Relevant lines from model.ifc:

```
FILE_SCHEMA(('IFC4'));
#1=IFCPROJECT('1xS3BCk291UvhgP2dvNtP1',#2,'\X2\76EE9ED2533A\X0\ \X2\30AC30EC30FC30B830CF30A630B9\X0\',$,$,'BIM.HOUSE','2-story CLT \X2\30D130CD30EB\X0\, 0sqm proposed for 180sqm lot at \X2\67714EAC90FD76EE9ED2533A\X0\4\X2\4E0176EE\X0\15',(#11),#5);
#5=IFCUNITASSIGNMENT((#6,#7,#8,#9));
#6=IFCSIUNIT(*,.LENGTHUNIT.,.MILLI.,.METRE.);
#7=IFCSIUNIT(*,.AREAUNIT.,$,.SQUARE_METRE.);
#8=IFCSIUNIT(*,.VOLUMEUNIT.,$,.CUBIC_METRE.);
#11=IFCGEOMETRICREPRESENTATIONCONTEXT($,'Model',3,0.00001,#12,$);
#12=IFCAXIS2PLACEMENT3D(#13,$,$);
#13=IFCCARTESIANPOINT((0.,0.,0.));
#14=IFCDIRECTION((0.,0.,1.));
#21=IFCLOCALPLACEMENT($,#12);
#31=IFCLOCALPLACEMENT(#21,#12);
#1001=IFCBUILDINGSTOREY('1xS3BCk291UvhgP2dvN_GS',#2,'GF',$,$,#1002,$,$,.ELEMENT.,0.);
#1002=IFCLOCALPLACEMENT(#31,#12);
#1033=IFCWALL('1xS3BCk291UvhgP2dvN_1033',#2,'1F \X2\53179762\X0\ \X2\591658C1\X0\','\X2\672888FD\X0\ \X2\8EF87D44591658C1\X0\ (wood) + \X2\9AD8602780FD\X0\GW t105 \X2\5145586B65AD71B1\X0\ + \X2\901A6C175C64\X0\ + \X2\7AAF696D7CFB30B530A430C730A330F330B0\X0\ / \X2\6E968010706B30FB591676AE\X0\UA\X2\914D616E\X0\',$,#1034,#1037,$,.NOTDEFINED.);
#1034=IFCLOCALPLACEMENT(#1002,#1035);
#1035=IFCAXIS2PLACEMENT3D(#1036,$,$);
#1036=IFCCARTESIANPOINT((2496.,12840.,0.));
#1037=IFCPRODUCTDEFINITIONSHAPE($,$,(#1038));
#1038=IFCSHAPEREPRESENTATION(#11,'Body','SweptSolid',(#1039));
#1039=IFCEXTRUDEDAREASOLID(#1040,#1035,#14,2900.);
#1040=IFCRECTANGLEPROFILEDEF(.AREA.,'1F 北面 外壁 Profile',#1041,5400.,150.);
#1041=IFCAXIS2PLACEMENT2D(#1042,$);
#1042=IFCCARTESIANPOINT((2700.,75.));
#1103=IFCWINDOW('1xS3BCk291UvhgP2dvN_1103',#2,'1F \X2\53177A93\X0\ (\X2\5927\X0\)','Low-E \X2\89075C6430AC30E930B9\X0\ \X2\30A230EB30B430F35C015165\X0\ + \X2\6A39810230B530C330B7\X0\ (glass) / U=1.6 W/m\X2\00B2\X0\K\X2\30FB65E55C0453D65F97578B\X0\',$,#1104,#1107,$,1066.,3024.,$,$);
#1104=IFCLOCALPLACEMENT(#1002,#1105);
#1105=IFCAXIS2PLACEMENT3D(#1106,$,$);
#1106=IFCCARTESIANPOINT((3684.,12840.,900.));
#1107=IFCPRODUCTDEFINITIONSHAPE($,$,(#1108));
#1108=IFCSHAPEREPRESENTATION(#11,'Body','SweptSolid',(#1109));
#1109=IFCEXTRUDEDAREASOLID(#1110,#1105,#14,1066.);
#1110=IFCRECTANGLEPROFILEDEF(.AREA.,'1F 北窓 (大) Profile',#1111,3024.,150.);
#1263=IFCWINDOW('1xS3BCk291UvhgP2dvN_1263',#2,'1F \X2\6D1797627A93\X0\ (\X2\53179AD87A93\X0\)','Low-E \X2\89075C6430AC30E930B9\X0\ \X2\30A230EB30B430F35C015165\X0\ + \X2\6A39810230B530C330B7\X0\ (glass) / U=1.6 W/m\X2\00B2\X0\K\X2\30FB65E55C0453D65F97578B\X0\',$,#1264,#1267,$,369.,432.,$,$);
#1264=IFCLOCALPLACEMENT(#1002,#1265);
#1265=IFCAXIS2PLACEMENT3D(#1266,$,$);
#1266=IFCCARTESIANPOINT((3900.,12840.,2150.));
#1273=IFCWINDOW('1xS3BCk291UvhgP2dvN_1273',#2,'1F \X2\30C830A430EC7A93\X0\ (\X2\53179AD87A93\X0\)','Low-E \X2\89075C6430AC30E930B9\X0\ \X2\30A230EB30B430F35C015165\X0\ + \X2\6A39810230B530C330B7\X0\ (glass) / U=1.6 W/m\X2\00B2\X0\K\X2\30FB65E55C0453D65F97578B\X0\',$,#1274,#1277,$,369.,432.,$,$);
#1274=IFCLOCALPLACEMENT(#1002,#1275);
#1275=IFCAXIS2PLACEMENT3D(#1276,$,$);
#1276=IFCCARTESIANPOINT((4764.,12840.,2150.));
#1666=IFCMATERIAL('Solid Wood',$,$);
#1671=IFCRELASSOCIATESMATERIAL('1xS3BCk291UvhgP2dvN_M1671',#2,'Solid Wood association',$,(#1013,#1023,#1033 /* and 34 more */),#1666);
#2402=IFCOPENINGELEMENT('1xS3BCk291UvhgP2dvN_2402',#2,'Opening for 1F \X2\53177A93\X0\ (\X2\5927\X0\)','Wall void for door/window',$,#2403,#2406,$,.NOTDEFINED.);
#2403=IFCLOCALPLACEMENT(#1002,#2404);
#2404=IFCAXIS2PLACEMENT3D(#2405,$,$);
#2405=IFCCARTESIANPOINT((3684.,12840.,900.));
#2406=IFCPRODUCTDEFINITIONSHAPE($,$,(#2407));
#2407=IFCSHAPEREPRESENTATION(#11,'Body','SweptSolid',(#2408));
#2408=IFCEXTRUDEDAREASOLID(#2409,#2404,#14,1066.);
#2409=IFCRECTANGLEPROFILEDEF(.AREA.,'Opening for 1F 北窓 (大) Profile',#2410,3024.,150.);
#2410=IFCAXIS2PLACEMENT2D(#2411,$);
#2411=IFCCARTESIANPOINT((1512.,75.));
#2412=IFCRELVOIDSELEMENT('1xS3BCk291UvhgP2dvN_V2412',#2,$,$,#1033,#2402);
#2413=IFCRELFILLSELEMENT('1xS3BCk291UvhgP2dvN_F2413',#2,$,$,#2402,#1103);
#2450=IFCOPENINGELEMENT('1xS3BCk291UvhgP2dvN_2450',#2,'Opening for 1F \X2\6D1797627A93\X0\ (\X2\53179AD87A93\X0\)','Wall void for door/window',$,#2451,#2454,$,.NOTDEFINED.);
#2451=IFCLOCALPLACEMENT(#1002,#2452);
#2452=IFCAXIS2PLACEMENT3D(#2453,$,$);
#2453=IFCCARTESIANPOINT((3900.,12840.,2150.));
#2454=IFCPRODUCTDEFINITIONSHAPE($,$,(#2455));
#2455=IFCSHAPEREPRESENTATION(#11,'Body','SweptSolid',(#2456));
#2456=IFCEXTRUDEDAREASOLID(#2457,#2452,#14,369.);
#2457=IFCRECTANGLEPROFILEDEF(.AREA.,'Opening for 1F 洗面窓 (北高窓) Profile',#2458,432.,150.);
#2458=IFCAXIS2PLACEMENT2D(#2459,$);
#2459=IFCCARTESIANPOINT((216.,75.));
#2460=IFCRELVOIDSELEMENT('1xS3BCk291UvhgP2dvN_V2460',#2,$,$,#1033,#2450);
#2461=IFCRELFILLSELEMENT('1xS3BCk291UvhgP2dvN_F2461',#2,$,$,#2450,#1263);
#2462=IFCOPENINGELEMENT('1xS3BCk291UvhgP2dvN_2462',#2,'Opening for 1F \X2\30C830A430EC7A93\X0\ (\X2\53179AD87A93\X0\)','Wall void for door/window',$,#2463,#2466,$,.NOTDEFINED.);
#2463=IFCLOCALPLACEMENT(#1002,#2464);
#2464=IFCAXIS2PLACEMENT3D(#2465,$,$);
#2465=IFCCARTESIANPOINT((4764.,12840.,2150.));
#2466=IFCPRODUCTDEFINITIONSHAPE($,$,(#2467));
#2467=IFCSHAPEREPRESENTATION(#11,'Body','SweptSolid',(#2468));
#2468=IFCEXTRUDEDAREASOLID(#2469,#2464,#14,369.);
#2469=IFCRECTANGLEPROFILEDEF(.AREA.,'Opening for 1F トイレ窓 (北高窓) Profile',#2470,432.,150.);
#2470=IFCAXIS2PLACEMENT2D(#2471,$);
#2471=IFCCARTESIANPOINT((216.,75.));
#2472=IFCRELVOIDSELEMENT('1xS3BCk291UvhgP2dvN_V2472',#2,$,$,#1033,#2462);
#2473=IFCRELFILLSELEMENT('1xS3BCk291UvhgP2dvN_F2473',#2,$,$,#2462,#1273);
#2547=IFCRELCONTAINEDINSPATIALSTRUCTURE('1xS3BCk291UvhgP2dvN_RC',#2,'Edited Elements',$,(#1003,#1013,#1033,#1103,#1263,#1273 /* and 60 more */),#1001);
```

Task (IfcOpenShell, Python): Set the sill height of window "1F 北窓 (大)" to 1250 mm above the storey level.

```python
import numpy as np
import ifcopenshell
import ifcopenshell.api.geometry
import ifcopenshell.geom
import ifcopenshell.util.element
import ifcopenshell.util.placement
import ifcopenshell.util.shape
import ifcopenshell.util.unit

model = ifcopenshell.open("model.ifc")
unit_scale = ifcopenshell.util.unit.calculate_unit_scale(model)

window = model.by_guid("1xS3BCk291UvhgP2dvN_1103")
opening = window.FillsVoids[0].RelatingOpeningElement
storey = ifcopenshell.util.element.get_container(window, ifc_class="IfcBuildingStorey")
level = ifcopenshell.util.placement.get_local_placement(storey.ObjectPlacement)[2, 3]

# The opening's origin need not be at the sill, so measure its lowest point.
shape = ifcopenshell.geom.create_shape(ifcopenshell.geom.settings(), opening)
bottom = ifcopenshell.util.shape.get_shape_bottom_elevation(shape, shape.geometry) / unit_scale
dz = level + 1250.0 - bottom

shift = np.array([0.0, 0.0, dz])
# The window is not placed relative to its opening, so move both.
for product in (opening, window):
    matrix = ifcopenshell.util.placement.get_local_placement(product.ObjectPlacement)
    matrix[:3, 3] += shift
    ifcopenshell.api.geometry.edit_object_placement(model, product=product, matrix=matrix, is_si=False)

print(f"moved by {dz * unit_scale:+.3f} m")

model.write("model_v2.ifc")
```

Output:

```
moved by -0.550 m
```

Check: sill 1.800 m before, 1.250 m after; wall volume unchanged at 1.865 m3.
